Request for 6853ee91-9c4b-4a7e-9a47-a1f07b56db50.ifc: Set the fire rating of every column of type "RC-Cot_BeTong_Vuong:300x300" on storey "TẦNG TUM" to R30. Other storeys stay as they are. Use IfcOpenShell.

First a look at what the model holds.

```python
import ifcopenshell
import ifcopenshell.util.element

model = ifcopenshell.open("6853ee91-9c4b-4a7e-9a47-a1f07b56db50.ifc")
print(model.schema)
storey = next(s for s in model.by_type("IfcBuildingStorey") if s.Name == "TẦNG TUM")
columns = [e for e in ifcopenshell.util.element.get_decomposition(storey) if e.is_a("IfcColumn")]
seen = {}
for e in columns:
    element_type = ifcopenshell.util.element.get_type(e)
    key = (element_type.Name if element_type != e and element_type else None, ifcopenshell.util.element.get_pset(e, "Pset_ColumnCommon", "FireRating"))
    seen[key] = seen.get(key, 0) + 1
for (name, value), count in sorted(seen.items(), key=str):
    print(count, "x", name, "|", value)
```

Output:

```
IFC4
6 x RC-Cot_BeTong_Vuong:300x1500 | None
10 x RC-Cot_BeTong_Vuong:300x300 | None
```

```python
import ifcopenshell
import ifcopenshell.api.pset
import ifcopenshell.util.element

model = ifcopenshell.open("6853ee91-9c4b-4a7e-9a47-a1f07b56db50.ifc")

storey = next(s for s in model.by_type("IfcBuildingStorey") if s.Name == "TẦNG TUM")
columns = [e for e in ifcopenshell.util.element.get_decomposition(storey) if e.is_a("IfcColumn")]

count = 0
for e in columns:
    element_type = ifcopenshell.util.element.get_type(e)
    if element_type in (None, e) or element_type.Name != "RC-Cot_BeTong_Vuong:300x300":
        continue
    # add_pset returns the element's existing set when there is one.
    pset = ifcopenshell.api.pset.add_pset(model, product=e, name="Pset_ColumnCommon")
    ifcopenshell.api.pset.edit_pset(model, pset=pset, properties={"FireRating": "R30"})
    count += 1

print(count, "columns updated")

model.write("6853ee91-9c4b-4a7e-9a47-a1f07b56db50_updated.ifc")
```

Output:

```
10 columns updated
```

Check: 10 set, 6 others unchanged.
